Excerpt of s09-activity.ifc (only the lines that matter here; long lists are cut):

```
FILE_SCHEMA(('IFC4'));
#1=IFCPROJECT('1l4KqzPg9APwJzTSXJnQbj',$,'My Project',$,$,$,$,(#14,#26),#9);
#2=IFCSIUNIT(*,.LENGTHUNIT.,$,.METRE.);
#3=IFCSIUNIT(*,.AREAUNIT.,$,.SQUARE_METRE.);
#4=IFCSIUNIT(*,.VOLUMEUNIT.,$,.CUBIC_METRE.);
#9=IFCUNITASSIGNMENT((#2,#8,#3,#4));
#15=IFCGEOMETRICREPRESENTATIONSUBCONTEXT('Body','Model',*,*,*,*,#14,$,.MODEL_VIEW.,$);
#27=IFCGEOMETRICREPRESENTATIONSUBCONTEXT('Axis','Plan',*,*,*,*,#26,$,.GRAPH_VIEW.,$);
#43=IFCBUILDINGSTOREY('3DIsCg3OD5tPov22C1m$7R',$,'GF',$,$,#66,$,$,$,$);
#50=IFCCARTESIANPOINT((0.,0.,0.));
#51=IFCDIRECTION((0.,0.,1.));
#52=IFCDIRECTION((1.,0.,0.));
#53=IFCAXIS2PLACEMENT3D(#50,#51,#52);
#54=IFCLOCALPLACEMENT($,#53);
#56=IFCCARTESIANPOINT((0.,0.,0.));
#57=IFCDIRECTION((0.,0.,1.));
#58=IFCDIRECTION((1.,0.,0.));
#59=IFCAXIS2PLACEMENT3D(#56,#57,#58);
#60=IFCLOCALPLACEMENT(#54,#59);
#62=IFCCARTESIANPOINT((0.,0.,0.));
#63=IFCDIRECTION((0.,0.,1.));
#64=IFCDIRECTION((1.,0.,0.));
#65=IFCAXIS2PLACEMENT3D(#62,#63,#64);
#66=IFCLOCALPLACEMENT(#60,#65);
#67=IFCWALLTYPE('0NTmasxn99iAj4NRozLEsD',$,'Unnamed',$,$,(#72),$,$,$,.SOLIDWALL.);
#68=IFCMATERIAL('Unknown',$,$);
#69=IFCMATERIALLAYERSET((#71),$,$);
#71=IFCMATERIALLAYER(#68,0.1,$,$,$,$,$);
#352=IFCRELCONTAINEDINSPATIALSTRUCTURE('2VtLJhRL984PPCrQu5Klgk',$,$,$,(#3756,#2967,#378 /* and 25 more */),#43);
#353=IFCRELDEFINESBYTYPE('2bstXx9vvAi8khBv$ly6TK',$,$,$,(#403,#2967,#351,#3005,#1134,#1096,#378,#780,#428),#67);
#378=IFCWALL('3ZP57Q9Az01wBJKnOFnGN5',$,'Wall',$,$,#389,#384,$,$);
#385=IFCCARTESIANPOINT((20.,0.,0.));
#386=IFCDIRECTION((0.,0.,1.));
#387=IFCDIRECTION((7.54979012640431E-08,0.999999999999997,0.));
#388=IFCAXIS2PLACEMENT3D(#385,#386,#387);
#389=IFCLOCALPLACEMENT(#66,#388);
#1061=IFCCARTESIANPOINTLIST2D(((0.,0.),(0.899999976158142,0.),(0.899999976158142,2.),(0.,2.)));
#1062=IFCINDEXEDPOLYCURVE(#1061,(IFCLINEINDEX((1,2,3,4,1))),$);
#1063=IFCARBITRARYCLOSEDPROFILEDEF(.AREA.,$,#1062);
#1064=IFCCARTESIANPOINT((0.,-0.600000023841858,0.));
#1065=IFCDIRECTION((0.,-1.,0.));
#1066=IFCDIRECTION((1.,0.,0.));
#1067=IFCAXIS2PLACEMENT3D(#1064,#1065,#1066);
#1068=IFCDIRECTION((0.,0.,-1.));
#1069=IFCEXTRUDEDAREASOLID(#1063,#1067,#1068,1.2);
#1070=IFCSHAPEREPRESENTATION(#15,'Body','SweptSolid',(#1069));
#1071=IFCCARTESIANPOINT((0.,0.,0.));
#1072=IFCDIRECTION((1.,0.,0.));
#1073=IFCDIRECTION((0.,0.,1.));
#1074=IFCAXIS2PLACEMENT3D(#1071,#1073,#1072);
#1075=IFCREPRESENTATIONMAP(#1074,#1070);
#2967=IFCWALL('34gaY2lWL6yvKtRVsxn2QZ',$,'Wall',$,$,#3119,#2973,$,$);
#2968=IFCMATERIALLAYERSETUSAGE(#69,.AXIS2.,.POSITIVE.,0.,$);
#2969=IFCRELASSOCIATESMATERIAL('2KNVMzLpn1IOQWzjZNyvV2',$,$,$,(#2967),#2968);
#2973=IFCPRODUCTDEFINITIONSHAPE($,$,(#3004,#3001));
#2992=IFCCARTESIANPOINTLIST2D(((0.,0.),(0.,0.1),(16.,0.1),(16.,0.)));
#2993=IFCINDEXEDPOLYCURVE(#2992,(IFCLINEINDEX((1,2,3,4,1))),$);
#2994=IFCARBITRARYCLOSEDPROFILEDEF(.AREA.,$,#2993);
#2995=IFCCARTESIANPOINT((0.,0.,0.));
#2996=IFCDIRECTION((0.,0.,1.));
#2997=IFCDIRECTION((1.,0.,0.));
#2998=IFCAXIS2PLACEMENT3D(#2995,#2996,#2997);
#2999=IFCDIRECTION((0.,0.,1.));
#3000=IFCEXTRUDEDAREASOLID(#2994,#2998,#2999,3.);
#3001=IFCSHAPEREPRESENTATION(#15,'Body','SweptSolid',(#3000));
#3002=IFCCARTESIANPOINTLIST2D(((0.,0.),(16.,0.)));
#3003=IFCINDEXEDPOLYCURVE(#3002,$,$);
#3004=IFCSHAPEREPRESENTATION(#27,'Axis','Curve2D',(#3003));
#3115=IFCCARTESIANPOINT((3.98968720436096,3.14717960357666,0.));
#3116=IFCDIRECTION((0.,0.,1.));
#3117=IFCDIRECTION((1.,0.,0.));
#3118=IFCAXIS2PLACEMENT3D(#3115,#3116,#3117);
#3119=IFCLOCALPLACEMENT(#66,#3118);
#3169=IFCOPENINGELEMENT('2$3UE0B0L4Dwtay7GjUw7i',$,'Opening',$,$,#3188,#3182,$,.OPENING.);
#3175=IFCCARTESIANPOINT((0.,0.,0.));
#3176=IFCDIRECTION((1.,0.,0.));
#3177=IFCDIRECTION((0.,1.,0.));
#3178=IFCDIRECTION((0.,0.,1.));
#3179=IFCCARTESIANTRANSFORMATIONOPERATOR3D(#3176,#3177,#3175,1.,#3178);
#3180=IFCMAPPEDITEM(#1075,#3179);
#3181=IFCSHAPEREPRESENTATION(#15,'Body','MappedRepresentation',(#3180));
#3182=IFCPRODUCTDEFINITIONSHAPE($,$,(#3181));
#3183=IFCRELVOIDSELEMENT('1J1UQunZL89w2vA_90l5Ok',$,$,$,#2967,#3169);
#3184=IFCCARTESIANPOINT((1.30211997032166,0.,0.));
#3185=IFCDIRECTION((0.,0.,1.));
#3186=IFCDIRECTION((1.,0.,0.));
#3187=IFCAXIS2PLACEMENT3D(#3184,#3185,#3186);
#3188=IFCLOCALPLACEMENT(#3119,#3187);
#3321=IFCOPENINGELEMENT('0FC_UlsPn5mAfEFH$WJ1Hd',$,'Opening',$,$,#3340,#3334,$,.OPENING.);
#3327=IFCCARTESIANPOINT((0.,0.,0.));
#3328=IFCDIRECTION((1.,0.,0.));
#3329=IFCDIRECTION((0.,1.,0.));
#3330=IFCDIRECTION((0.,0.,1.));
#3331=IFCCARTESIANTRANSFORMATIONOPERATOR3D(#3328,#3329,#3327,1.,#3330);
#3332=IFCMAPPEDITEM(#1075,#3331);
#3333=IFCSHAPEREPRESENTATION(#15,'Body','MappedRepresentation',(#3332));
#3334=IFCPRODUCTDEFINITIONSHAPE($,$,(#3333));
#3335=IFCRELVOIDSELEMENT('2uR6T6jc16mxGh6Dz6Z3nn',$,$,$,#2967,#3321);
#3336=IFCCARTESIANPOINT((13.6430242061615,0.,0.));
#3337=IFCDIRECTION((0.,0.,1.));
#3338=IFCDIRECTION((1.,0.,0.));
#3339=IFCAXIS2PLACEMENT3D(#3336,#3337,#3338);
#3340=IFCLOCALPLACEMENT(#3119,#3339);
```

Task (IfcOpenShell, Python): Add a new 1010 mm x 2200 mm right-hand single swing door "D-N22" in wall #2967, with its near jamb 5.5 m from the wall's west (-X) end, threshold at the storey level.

```python
import numpy as np
import ifcopenshell
import ifcopenshell.api.feature
import ifcopenshell.api.geometry
import ifcopenshell.api.root
import ifcopenshell.api.spatial
import ifcopenshell.geom
import ifcopenshell.util.element
import ifcopenshell.util.placement
import ifcopenshell.util.representation
import ifcopenshell.util.shape
import ifcopenshell.util.unit

model = ifcopenshell.open("s09-activity.ifc")
unit_scale = ifcopenshell.util.unit.calculate_unit_scale(model)
settings = ifcopenshell.geom.settings()


def volume(element):
    """Net volume in cubic metres, openings subtracted."""
    shape = ifcopenshell.geom.create_shape(settings, element)
    return ifcopenshell.util.shape.get_volume(shape.geometry)


wall = model.by_id(2967)
storey = ifcopenshell.util.element.get_container(wall, ifc_class="IfcBuildingStorey")
context = ifcopenshell.util.representation.get_context(model, "Model", "Body", "MODEL_VIEW")
before = volume(wall)

width, height, from_end, sill = 1.01, 2.2, 5.5, 0.0  # metres

# The wall runs along its own X axis, and the end named is its -X end.
wall_shape = ifcopenshell.geom.create_shape(settings, wall)
x, y, z = ifcopenshell.util.shape.get_vertices(wall_shape.geometry).T
start = x.min() + from_end
face, thickness = float(y.min()), float(y.max() - y.min())
wall_matrix = ifcopenshell.util.placement.get_local_placement(wall.ObjectPlacement)
level = ifcopenshell.util.placement.get_local_placement(storey.ObjectPlacement)[2, 3]


def in_wall(x, y):
    """Placement at x, y metres in the wall's axes, at sill height."""
    matrix = wall_matrix.copy()
    matrix[:, 3] = wall_matrix @ np.array([x / unit_scale, y / unit_scale, 0.0, 1.0])
    matrix[2, 3] = level + sill / unit_scale
    return matrix


# Opening: a box that overshoots both wall faces by 50 mm.
opening = ifcopenshell.api.root.create_entity(model, ifc_class="IfcOpeningElement", predefined_type="OPENING")
box = ifcopenshell.api.geometry.add_wall_representation(
    model, context=context, length=width, height=height, thickness=thickness + 0.1
)
ifcopenshell.api.geometry.assign_representation(model, product=opening, representation=box)
ifcopenshell.api.geometry.edit_object_placement(model, product=opening, matrix=in_wall(start, face - 0.05), is_si=False)
ifcopenshell.api.feature.add_feature(model, feature=opening, element=wall)

door = ifcopenshell.api.root.create_entity(model, ifc_class="IfcDoor", name="D-N22", predefined_type="DOOR")
door.OverallWidth, door.OverallHeight = width / unit_scale, height / unit_scale
door.OperationType = "SINGLE_SWING_RIGHT"
body = ifcopenshell.api.geometry.add_door_representation(
    model,
    context=context,
    overall_width=door.OverallWidth,
    overall_height=door.OverallHeight,
    operation_type="SINGLE_SWING_RIGHT",
    lining_properties={"LiningDepth": thickness / unit_scale, "ThresholdDepth": thickness / unit_scale},
)
ifcopenshell.api.geometry.assign_representation(model, product=door, representation=body)
ifcopenshell.api.spatial.assign_container(model, products=[door], relating_structure=storey)
ifcopenshell.api.feature.add_filling(model, opening=opening, element=door)

# The lining spans the wall, so the door starts at the wall face.
ifcopenshell.api.geometry.edit_object_placement(model, product=door, matrix=in_wall(start, face), is_si=False)

after = volume(wall)

print(f"wall volume {before:.3f} -> {after:.3f} m3")

model.write("s09-activity_rev.ifc")
```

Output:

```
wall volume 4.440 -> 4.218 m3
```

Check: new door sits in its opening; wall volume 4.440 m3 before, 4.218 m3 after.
